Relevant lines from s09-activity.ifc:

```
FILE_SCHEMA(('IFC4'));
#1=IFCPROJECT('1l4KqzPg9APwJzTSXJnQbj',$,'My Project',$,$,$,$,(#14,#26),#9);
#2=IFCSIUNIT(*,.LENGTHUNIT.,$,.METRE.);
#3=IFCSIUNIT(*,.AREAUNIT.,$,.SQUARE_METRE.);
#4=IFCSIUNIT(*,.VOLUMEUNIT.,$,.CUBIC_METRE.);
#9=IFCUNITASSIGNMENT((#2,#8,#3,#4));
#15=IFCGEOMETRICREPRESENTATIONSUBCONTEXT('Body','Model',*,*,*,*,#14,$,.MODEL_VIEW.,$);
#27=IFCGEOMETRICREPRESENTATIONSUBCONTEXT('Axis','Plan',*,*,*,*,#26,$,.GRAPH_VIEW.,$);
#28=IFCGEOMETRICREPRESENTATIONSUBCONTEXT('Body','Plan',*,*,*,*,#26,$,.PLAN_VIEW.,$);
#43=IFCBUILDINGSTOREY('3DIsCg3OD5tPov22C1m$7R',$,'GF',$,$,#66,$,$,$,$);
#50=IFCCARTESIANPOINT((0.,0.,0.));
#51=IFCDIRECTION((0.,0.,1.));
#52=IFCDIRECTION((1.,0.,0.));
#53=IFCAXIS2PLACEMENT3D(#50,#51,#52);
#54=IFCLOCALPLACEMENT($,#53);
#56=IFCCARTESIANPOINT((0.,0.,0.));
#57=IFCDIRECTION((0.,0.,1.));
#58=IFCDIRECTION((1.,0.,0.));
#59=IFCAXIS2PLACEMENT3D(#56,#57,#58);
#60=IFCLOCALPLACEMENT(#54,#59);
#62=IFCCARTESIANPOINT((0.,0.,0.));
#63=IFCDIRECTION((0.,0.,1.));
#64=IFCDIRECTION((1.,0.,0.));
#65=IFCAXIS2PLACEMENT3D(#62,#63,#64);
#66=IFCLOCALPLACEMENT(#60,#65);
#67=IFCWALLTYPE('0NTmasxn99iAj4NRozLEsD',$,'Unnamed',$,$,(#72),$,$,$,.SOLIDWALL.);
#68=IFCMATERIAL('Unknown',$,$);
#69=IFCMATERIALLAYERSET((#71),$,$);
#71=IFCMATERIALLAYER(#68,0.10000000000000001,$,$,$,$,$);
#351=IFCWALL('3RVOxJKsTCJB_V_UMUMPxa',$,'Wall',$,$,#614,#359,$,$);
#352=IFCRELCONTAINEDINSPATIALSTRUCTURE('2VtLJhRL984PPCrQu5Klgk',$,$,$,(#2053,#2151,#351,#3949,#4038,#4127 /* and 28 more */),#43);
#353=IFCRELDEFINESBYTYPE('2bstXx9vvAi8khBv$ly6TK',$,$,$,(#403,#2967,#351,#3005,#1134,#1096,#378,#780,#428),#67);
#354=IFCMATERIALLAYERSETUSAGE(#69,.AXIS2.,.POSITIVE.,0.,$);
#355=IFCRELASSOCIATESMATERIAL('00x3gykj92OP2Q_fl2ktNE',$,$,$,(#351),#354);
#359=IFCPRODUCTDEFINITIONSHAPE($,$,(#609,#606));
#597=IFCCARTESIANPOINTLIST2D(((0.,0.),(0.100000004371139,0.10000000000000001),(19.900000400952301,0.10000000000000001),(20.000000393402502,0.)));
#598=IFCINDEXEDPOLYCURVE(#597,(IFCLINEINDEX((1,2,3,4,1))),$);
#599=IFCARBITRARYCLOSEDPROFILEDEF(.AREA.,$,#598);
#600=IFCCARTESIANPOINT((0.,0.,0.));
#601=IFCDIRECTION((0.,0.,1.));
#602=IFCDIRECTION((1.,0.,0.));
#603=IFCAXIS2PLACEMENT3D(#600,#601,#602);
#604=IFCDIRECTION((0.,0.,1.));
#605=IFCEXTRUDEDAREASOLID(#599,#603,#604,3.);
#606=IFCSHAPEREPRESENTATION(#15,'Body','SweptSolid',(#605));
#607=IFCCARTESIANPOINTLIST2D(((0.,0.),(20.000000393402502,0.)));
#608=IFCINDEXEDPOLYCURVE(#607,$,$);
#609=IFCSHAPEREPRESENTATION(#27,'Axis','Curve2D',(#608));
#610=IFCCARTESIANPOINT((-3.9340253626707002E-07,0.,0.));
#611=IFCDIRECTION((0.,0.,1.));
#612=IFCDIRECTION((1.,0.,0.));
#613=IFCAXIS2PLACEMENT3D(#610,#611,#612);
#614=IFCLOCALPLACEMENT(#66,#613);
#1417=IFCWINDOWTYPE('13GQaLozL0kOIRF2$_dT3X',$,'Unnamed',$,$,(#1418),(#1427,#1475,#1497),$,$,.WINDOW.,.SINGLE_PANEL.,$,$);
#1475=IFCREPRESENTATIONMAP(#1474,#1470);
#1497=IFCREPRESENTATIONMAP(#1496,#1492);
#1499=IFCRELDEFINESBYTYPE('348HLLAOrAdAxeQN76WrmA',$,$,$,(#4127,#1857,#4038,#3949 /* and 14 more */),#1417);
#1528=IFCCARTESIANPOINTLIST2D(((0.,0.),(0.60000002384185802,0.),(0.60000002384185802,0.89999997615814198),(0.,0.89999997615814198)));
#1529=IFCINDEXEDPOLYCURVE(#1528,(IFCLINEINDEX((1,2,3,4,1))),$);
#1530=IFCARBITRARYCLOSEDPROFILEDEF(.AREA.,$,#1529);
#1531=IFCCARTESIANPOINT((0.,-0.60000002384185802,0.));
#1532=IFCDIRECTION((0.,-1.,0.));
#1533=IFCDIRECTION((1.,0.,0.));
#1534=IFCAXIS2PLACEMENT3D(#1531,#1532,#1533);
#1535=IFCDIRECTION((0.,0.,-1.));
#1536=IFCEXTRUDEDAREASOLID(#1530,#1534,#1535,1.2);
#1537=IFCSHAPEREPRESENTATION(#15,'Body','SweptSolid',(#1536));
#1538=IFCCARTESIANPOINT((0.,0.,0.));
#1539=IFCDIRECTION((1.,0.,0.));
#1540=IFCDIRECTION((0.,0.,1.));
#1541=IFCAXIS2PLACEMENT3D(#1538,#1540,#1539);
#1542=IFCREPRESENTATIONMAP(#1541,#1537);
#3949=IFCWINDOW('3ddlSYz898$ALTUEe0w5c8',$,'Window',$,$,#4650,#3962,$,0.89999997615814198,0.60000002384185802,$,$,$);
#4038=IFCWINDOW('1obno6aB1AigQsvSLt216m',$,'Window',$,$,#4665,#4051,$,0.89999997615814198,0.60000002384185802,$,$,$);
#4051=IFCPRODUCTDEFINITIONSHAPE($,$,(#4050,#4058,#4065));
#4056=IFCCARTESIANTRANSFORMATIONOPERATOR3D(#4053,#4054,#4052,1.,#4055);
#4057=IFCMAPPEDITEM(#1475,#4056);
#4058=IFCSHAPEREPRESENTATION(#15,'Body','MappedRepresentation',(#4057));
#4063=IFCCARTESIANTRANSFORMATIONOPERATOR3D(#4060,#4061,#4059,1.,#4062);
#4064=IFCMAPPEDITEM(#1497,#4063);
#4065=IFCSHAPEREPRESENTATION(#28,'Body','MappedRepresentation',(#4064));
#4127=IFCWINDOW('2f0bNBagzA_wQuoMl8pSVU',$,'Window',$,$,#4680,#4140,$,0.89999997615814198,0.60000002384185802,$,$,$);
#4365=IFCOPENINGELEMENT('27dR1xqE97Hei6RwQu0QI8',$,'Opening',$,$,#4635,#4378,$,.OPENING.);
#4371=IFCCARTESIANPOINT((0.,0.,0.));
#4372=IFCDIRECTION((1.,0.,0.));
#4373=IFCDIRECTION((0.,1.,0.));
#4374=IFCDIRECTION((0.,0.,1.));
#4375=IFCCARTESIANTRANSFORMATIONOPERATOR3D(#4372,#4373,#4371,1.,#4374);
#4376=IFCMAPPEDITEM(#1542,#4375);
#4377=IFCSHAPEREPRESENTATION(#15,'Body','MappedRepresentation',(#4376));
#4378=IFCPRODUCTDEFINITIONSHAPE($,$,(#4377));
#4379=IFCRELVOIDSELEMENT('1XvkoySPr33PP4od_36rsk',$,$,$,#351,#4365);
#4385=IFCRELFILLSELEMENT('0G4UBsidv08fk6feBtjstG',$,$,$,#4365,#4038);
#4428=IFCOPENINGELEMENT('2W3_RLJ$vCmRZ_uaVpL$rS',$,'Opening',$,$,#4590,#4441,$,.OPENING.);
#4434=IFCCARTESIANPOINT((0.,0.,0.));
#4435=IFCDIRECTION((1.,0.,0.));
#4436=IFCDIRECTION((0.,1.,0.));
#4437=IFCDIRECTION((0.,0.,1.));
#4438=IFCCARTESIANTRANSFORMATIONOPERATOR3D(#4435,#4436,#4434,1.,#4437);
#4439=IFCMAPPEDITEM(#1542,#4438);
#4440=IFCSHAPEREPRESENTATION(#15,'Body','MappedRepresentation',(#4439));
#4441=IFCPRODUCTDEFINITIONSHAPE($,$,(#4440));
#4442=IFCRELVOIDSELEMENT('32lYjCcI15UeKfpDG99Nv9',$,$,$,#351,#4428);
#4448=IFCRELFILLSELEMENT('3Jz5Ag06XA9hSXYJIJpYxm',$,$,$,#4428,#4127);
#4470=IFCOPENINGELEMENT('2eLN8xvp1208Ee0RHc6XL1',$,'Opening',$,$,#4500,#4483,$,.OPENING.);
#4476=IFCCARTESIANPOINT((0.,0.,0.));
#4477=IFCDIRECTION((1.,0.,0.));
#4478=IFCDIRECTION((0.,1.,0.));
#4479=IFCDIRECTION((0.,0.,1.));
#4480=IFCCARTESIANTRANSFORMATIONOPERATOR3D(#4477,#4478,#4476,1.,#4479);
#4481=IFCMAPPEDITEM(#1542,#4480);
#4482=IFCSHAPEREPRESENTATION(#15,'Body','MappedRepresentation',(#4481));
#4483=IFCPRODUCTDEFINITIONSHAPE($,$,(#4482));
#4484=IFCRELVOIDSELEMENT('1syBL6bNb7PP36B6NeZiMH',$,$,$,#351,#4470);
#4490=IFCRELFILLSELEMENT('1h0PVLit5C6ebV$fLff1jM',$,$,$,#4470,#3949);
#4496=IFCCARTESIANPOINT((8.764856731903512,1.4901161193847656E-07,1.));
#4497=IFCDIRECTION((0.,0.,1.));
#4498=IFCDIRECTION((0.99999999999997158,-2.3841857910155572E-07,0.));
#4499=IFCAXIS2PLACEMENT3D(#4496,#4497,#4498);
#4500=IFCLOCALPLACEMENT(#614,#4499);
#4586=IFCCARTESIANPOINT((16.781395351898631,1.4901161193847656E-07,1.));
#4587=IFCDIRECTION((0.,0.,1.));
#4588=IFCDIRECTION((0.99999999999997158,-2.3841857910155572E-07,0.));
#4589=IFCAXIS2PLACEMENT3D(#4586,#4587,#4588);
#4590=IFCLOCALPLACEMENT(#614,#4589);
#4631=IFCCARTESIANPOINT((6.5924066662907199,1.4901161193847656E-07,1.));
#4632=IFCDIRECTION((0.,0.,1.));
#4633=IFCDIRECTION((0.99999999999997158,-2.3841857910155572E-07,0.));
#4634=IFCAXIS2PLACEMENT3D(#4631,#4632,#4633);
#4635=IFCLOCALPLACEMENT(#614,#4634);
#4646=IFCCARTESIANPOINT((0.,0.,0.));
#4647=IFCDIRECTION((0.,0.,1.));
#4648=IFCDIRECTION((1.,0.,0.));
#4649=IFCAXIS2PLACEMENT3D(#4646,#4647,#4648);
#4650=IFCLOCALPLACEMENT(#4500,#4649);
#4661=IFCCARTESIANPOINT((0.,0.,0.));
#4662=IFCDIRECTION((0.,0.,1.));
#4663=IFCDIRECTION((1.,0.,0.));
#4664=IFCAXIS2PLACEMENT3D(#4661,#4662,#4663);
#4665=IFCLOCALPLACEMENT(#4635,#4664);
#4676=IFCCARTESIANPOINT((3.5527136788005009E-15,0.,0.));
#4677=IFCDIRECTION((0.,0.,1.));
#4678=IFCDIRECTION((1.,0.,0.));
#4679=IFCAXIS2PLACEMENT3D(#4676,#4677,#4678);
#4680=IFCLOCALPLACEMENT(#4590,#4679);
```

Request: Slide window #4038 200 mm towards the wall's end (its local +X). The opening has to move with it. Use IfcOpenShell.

```python
import ifcopenshell
import ifcopenshell.api.geometry
import ifcopenshell.util.placement
import ifcopenshell.util.unit

model = ifcopenshell.open("s09-activity.ifc")
unit_scale = ifcopenshell.util.unit.calculate_unit_scale(model)

window = model.by_guid("1obno6aB1AigQsvSLt216m")
opening = window.FillsVoids[0].RelatingOpeningElement
wall = opening.VoidsElements[0].RelatingBuildingElement

wall_matrix = ifcopenshell.util.placement.get_local_placement(wall.ObjectPlacement)
shift = wall_matrix[:3, 0] * 0.2 / unit_scale
before = ifcopenshell.util.placement.get_local_placement(window.ObjectPlacement)[:3, 3].copy()

# The window is placed relative to its opening, so it follows when the opening moves.
matrix = ifcopenshell.util.placement.get_local_placement(opening.ObjectPlacement)
matrix[:3, 3] += shift
ifcopenshell.api.geometry.edit_object_placement(
    model, product=opening, matrix=matrix, is_si=False, should_transform_children=True
)

after = ifcopenshell.util.placement.get_local_placement(window.ObjectPlacement)[:3, 3]
print("window moved by", (after - before).round(3) + 0.0)

model.write("s09-activity_updated.ifc")
```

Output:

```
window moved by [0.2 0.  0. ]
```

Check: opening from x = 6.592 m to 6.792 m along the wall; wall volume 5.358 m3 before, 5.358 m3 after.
